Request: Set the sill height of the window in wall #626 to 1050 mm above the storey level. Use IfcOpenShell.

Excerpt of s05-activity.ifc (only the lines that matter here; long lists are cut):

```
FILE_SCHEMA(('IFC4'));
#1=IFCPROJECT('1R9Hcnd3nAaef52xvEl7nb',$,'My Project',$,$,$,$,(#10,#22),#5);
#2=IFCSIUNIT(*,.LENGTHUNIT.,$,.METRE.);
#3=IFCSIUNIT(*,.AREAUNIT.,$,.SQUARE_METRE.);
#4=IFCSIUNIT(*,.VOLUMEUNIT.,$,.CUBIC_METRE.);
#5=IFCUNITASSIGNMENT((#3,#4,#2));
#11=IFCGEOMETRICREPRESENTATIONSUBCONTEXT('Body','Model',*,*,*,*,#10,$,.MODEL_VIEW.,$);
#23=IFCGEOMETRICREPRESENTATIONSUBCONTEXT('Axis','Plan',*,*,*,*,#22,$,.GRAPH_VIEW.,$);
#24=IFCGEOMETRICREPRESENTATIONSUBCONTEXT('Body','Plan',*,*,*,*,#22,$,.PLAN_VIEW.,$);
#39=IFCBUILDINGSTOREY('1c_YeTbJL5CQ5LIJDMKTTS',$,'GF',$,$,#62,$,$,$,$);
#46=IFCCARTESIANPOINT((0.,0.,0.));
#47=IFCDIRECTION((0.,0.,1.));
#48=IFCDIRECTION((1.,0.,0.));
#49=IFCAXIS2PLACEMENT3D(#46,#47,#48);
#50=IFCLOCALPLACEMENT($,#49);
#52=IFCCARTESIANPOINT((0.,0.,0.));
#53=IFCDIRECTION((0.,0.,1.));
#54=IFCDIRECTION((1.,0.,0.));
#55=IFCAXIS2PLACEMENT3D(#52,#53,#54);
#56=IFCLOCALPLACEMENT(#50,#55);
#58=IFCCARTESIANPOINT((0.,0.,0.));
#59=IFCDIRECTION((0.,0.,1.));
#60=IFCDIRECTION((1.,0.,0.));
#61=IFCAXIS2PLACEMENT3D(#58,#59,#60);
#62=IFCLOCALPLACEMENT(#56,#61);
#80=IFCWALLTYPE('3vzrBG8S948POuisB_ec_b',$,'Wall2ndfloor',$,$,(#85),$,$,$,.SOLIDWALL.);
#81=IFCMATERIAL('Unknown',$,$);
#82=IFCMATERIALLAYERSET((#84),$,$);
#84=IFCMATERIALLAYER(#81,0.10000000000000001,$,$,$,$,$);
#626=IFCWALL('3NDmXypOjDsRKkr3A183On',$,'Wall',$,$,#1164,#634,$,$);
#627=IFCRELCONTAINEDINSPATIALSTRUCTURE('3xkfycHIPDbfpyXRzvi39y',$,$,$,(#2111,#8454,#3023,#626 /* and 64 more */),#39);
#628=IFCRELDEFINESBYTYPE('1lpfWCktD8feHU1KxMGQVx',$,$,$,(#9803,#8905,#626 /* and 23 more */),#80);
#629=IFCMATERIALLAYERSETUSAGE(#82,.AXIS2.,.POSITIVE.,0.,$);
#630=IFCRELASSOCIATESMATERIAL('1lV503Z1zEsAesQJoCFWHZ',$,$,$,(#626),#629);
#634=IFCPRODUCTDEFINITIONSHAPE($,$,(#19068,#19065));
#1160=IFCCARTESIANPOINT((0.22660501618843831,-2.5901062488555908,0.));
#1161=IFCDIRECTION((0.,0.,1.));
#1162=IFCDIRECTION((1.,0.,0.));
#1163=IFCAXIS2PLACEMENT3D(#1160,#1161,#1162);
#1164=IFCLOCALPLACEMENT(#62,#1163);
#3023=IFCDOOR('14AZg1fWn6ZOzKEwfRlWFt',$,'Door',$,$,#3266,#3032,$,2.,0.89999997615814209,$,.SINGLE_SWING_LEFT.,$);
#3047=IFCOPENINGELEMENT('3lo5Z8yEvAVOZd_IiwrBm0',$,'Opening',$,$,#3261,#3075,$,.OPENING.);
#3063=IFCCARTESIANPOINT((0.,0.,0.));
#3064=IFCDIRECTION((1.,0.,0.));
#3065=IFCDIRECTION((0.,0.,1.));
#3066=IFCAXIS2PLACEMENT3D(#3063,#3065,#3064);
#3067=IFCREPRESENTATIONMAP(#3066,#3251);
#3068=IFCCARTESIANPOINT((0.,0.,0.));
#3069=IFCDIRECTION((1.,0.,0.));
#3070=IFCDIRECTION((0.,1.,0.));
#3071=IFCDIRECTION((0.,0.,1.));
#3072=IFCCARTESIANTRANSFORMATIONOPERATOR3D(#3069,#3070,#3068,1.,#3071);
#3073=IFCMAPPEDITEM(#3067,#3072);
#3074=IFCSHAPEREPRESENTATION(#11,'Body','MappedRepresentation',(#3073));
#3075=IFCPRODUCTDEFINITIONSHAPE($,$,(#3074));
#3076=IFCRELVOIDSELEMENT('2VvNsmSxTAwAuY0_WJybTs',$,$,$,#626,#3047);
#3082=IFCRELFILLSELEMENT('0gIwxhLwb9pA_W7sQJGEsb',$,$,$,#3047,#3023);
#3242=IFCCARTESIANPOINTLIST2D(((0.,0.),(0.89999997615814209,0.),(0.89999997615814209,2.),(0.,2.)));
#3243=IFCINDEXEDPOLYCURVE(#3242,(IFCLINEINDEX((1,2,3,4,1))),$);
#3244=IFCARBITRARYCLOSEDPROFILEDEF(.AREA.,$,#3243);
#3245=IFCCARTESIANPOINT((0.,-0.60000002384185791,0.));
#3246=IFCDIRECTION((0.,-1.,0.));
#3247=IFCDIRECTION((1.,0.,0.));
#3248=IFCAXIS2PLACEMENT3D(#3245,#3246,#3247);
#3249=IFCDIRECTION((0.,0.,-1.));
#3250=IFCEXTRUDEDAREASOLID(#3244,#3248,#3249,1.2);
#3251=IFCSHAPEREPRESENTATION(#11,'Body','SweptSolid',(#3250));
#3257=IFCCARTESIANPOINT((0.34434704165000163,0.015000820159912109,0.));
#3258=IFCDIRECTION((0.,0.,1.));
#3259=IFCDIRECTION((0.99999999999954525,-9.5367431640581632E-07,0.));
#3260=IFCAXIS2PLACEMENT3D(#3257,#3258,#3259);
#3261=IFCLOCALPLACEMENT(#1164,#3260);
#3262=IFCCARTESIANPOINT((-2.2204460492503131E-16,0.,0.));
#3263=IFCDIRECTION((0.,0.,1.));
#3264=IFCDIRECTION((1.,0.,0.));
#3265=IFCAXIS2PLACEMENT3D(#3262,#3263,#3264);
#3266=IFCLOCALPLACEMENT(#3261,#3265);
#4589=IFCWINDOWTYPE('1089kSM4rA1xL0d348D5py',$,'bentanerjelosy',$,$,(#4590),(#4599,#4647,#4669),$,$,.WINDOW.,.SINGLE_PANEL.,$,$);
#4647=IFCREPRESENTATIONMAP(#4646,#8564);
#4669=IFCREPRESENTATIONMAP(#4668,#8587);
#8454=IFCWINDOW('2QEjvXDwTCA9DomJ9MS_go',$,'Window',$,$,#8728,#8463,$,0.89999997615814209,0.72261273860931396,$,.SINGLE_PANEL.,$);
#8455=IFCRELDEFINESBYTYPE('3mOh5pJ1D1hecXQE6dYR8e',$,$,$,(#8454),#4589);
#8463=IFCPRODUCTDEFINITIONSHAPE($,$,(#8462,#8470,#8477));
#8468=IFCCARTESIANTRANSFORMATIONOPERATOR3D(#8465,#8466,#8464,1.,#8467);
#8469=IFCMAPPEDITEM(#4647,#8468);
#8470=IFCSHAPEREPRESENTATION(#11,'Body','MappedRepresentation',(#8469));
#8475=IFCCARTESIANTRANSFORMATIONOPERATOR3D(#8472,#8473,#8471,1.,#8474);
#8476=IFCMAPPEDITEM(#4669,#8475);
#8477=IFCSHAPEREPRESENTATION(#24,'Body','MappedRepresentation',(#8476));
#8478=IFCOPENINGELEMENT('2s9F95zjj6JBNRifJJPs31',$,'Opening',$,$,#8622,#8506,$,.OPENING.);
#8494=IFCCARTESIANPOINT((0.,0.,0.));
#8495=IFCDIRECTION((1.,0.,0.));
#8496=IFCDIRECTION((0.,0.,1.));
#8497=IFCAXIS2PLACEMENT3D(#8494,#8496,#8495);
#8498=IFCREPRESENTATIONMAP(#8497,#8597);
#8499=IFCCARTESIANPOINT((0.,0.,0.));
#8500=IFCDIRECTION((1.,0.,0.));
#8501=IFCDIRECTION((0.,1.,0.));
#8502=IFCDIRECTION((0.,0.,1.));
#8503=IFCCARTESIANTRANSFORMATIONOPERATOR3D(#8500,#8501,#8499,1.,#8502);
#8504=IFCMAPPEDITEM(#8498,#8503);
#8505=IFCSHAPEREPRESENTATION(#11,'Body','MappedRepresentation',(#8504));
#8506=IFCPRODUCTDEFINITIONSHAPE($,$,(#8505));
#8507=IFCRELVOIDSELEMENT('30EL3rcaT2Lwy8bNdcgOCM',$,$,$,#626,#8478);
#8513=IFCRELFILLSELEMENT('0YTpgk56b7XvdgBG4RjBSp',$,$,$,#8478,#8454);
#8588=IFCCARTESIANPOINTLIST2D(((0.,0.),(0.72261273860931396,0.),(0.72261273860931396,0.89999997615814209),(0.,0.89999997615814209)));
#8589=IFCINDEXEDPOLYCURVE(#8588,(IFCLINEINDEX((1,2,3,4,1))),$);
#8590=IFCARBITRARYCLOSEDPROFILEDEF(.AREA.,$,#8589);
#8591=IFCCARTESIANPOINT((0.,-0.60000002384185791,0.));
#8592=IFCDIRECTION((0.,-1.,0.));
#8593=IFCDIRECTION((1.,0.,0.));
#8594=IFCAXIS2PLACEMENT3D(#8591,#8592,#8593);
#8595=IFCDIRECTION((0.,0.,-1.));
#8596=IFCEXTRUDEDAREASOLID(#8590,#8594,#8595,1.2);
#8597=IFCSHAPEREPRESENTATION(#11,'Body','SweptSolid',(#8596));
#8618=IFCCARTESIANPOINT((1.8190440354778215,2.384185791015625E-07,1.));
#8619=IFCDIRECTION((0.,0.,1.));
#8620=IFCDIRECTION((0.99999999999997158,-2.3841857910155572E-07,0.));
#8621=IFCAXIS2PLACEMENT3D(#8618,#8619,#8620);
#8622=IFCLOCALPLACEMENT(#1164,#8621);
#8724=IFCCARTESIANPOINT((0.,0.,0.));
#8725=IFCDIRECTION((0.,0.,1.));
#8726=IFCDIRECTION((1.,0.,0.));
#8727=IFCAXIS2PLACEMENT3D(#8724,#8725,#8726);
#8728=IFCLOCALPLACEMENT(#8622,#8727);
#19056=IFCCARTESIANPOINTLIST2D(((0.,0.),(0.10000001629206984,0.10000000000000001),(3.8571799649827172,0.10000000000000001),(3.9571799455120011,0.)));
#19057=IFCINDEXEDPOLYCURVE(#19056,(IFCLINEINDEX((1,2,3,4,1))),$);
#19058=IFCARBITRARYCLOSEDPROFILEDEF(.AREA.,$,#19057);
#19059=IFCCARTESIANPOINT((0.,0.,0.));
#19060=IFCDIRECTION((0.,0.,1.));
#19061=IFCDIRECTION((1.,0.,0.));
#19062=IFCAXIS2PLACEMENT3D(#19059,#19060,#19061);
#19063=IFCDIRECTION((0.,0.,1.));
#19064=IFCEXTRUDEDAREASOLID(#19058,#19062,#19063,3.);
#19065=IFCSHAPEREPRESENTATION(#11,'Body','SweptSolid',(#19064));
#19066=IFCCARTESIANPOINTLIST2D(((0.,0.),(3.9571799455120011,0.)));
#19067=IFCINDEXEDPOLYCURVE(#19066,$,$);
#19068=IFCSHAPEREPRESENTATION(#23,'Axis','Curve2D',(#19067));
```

```python
import numpy as np
import ifcopenshell
import ifcopenshell.api.geometry
import ifcopenshell.geom
import ifcopenshell.util.element
import ifcopenshell.util.placement
import ifcopenshell.util.shape
import ifcopenshell.util.unit

model = ifcopenshell.open("s05-activity.ifc")
unit_scale = ifcopenshell.util.unit.calculate_unit_scale(model)

window = model.by_guid("2QEjvXDwTCA9DomJ9MS_go")
opening = window.FillsVoids[0].RelatingOpeningElement
storey = ifcopenshell.util.element.get_container(window, ifc_class="IfcBuildingStorey")
level = ifcopenshell.util.placement.get_local_placement(storey.ObjectPlacement)[2, 3]

# The opening's origin need not be at the sill, so measure its lowest point.
shape = ifcopenshell.geom.create_shape(ifcopenshell.geom.settings(), opening)
bottom = ifcopenshell.util.shape.get_shape_bottom_elevation(shape, shape.geometry) / unit_scale
dz = level + 1.05 / unit_scale - bottom

shift = np.array([0.0, 0.0, dz])
# The window is placed relative to its opening, so it follows when the opening moves.
matrix = ifcopenshell.util.placement.get_local_placement(opening.ObjectPlacement)
matrix[:3, 3] += shift
ifcopenshell.api.geometry.edit_object_placement(
    model, product=opening, matrix=matrix, is_si=False, should_transform_children=True
)

print(f"moved by {dz * unit_scale:+.3f} m")

model.write("s05-activity-out.ifc")
```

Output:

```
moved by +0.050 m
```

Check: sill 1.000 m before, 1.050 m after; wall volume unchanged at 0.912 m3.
